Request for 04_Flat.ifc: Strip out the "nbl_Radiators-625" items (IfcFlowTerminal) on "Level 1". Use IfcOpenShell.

First a look at what the model holds.

```python
import ifcopenshell
import ifcopenshell.util.element

model = ifcopenshell.open("04_Flat.ifc")
print(model.schema)
storey = next(s for s in model.by_type("IfcBuildingStorey") if s.Name == "Level 1")
terminals = [e for e in ifcopenshell.util.element.get_decomposition(storey) if e.is_a("IfcFlowTerminal")]
seen = {}
for e in terminals:
    element_type = ifcopenshell.util.element.get_type(e)
    name = element_type.Name if element_type not in (None, e) else None
    seen[name] = seen.get(name, 0) + 1
for name, count in sorted(seen.items(), key=str):
    print(count, "x", name)
```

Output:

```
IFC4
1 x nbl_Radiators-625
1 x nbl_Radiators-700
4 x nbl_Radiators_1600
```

```python
import ifcopenshell
import ifcopenshell.api.root
import ifcopenshell.util.element

model = ifcopenshell.open("04_Flat.ifc")

storey = next(s for s in model.by_type("IfcBuildingStorey") if s.Name == "Level 1")
terminals = [e for e in ifcopenshell.util.element.get_decomposition(storey) if e.is_a("IfcFlowTerminal")]
targets = [e for e in terminals if (t := ifcopenshell.util.element.get_type(e)) not in (None, e) and t.Name == "nbl_Radiators-625"]

for e in targets:
    ifcopenshell.api.root.remove_product(model, product=e)
print(len(targets), "removed")

model.write("04_Flat_updated.ifc")
```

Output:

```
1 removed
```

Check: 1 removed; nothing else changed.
